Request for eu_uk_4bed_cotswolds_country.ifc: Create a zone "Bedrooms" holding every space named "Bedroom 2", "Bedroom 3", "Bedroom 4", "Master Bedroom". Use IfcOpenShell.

First a look at what the model holds.

```python
import ifcopenshell

model = ifcopenshell.open("eu_uk_4bed_cotswolds_country.ifc")
print(model.schema)
seen = {}
for space in model.by_type("IfcSpace"):
    seen[space.LongName] = seen.get(space.LongName, 0) + 1
for name, count in sorted(seen.items(), key=str):
    print(count, "x", name)
print("zones:", [z.Name for z in model.by_type("IfcZone")][:20])
```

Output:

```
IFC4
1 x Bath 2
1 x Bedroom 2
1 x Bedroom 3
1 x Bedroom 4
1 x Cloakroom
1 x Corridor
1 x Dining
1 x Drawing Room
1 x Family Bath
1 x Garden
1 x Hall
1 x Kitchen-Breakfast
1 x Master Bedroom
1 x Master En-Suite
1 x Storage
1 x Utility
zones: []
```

```python
import ifcopenshell
import ifcopenshell.api.group
import ifcopenshell.api.root

model = ifcopenshell.open("eu_uk_4bed_cotswolds_country.ifc")

names = {"Bedroom 2", "Bedroom 3", "Bedroom 4", "Master Bedroom"}
spaces = [s for s in model.by_type("IfcSpace") if s.LongName in names]

zone = ifcopenshell.api.root.create_entity(model, ifc_class="IfcZone", name="Bedrooms")
ifcopenshell.api.group.assign_group(model, products=spaces, group=zone)
print(len(spaces), "spaces in", zone.Name)

model.write("eu_uk_4bed_cotswolds_country_rev.ifc")
```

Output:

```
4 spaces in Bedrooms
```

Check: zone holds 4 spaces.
